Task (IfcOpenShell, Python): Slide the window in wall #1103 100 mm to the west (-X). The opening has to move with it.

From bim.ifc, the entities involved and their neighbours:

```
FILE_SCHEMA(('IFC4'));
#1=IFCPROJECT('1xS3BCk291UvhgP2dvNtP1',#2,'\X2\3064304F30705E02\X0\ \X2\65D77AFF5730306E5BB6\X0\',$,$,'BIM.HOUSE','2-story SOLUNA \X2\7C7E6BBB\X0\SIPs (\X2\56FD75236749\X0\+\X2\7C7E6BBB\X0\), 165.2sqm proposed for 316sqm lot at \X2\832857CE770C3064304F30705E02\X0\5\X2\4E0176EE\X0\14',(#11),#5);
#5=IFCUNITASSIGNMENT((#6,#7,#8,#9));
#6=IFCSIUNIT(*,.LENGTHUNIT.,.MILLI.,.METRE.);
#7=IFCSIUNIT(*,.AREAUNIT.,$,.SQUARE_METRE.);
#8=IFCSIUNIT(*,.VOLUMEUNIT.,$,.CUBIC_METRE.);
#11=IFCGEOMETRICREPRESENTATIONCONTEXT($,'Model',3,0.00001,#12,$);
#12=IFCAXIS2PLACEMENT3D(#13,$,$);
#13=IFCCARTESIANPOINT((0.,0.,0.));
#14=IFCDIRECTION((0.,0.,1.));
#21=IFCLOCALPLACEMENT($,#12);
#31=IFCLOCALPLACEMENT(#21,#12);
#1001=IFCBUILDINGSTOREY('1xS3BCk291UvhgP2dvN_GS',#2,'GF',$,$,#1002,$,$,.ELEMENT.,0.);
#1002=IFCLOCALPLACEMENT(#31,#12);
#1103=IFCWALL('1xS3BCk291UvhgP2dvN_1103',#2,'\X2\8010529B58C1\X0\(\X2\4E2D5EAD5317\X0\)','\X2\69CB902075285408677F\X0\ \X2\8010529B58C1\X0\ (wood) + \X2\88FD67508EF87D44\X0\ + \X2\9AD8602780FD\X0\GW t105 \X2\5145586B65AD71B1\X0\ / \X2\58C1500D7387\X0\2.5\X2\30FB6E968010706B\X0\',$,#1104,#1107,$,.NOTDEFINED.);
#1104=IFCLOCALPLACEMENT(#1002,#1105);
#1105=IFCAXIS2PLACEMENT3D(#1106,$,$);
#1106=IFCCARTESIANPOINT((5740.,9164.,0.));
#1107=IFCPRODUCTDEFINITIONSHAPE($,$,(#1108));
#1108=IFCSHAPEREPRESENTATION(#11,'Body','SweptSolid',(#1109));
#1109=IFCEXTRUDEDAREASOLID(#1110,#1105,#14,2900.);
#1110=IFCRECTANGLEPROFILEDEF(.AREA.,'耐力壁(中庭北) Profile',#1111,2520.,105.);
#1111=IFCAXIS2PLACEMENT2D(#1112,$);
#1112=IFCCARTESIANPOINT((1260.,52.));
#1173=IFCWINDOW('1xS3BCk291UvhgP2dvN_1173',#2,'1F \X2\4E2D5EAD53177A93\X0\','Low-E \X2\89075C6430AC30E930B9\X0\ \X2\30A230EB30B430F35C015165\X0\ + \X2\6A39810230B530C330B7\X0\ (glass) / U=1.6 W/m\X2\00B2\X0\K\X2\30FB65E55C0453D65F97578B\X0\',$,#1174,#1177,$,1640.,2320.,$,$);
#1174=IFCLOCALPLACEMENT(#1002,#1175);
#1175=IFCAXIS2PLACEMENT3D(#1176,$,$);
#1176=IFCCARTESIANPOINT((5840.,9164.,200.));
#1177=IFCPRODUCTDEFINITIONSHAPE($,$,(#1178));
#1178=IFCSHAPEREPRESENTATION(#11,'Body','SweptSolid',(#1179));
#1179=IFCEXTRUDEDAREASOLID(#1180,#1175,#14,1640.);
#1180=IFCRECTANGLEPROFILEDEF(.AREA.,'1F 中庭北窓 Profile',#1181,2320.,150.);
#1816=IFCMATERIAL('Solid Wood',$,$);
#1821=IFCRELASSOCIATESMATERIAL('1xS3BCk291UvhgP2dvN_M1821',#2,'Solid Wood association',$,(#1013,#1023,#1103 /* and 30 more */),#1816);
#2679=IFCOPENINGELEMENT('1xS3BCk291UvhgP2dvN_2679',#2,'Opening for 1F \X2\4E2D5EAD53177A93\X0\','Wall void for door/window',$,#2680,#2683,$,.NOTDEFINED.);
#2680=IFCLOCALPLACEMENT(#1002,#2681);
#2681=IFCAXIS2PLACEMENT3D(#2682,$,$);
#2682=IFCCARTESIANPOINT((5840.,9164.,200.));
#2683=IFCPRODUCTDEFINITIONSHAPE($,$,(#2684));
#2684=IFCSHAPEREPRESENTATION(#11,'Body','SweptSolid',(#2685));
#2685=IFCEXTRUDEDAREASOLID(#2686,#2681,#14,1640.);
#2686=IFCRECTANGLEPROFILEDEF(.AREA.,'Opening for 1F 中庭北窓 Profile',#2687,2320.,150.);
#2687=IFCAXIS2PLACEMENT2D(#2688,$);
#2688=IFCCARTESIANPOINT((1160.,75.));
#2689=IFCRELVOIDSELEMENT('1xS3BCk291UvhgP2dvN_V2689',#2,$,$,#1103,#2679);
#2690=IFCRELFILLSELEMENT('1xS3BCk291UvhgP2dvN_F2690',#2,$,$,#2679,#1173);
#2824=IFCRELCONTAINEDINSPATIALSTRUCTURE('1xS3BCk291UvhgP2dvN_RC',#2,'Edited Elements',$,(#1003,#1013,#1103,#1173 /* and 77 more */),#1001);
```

```python
import ifcopenshell
import ifcopenshell.api.geometry
import ifcopenshell.util.placement

model = ifcopenshell.open("bim.ifc")

window = model.by_id(1173)
opening = window.FillsVoids[0].RelatingOpeningElement
wall = opening.VoidsElements[0].RelatingBuildingElement

wall_matrix = ifcopenshell.util.placement.get_local_placement(wall.ObjectPlacement)
shift = wall_matrix[:3, 0] * -100.0
before = ifcopenshell.util.placement.get_local_placement(window.ObjectPlacement)[:3, 3].copy()

# The window is not placed relative to its opening, so move both.
for product in (opening, window):
    matrix = ifcopenshell.util.placement.get_local_placement(product.ObjectPlacement)
    matrix[:3, 3] += shift
    ifcopenshell.api.geometry.edit_object_placement(model, product=product, matrix=matrix, is_si=False)

after = ifcopenshell.util.placement.get_local_placement(window.ObjectPlacement)[:3, 3]
print("window moved by", (after - before).round(3) + 0.0)

model.write("bim_updated.ifc")
```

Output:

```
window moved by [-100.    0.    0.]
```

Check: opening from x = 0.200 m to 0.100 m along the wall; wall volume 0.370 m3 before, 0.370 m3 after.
